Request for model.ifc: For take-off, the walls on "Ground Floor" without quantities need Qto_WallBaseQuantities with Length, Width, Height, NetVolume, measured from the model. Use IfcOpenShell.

First a look at what the model holds.

```python
import ifcopenshell
import ifcopenshell.util.element
import ifcopenshell.util.unit

model = ifcopenshell.open("model.ifc")
print(model.schema)
for unit_type in ("LENGTHUNIT", "AREAUNIT", "VOLUMEUNIT"):
    print(unit_type, ifcopenshell.util.unit.calculate_unit_scale(model, unit_type))
storey = next(s for s in model.by_type("IfcBuildingStorey") if s.Name == "Ground Floor")
walls = [e for e in ifcopenshell.util.element.get_decomposition(storey) if e.is_a("IfcWall")]
for e in sorted(walls, key=lambda e: e.id()):
    print(e.id(), e.is_a(), e.Name, list(ifcopenshell.util.element.get_psets(e, qtos_only=True)), sep=" | ")
```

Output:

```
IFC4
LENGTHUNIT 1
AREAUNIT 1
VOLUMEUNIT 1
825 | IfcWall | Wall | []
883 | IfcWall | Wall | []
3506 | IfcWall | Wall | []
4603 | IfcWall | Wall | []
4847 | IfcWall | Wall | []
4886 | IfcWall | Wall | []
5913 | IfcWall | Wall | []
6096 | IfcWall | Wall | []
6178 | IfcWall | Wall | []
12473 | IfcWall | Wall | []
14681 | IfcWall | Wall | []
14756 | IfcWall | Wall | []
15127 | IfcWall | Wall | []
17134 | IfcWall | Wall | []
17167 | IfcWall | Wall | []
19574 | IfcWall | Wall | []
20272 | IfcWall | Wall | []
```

```python
import ifcopenshell
import ifcopenshell.api.pset
import ifcopenshell.geom
import ifcopenshell.util.element
import ifcopenshell.util.shape
import ifcopenshell.util.unit

model = ifcopenshell.open("model.ifc")
unit_scale = ifcopenshell.util.unit.calculate_unit_scale(model)
volume_scale = ifcopenshell.util.unit.calculate_unit_scale(model, "VOLUMEUNIT")
settings = ifcopenshell.geom.settings()

storey = next(s for s in model.by_type("IfcBuildingStorey") if s.Name == "Ground Floor")
walls = [e for e in ifcopenshell.util.element.get_decomposition(storey) if e.is_a("IfcWall")]

for e in sorted(walls, key=lambda e: e.id()):
    if ifcopenshell.util.element.get_psets(e, qtos_only=True, should_inherit=False):
        continue
    # Geometry comes back in metres, in the element's own axes.
    shape = ifcopenshell.geom.create_shape(settings, e)
    values = {
        "Length": ifcopenshell.util.shape.get_x(shape.geometry) / unit_scale,
        "Width": ifcopenshell.util.shape.get_y(shape.geometry) / unit_scale,
        "Height": ifcopenshell.util.shape.get_z(shape.geometry) / unit_scale,
        "NetVolume": ifcopenshell.util.shape.get_volume(shape.geometry) / volume_scale,
    }
    qto = ifcopenshell.api.pset.add_qto(model, product=e, name="Qto_WallBaseQuantities")
    ifcopenshell.api.pset.edit_qto(model, qto=qto, properties=values)
    print(e.id(), {k: round(v, 3) for k, v in values.items()})

model.write("model_rev.ifc")
```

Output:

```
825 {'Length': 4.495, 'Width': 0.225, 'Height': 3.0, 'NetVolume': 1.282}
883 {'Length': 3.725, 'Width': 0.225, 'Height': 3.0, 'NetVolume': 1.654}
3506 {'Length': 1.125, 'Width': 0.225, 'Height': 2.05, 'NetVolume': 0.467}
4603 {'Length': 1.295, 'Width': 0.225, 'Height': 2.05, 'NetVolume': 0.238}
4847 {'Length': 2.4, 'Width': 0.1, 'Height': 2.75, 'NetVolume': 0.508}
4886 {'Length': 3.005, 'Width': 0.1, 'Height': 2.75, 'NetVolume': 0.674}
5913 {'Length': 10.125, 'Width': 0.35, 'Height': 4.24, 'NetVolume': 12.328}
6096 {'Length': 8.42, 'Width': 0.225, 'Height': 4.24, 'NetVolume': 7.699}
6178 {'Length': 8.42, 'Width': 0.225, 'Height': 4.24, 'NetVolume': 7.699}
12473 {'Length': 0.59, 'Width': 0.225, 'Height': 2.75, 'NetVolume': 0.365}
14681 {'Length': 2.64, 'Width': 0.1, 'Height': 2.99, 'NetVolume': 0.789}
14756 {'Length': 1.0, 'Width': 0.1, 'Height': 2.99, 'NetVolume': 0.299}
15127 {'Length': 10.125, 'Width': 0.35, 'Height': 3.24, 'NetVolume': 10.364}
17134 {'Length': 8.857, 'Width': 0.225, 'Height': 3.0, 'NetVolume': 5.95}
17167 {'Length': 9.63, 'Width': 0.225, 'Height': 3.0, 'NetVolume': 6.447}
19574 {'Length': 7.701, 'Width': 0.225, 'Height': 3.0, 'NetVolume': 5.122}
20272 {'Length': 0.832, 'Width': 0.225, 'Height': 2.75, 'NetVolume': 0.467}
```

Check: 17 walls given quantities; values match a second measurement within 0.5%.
